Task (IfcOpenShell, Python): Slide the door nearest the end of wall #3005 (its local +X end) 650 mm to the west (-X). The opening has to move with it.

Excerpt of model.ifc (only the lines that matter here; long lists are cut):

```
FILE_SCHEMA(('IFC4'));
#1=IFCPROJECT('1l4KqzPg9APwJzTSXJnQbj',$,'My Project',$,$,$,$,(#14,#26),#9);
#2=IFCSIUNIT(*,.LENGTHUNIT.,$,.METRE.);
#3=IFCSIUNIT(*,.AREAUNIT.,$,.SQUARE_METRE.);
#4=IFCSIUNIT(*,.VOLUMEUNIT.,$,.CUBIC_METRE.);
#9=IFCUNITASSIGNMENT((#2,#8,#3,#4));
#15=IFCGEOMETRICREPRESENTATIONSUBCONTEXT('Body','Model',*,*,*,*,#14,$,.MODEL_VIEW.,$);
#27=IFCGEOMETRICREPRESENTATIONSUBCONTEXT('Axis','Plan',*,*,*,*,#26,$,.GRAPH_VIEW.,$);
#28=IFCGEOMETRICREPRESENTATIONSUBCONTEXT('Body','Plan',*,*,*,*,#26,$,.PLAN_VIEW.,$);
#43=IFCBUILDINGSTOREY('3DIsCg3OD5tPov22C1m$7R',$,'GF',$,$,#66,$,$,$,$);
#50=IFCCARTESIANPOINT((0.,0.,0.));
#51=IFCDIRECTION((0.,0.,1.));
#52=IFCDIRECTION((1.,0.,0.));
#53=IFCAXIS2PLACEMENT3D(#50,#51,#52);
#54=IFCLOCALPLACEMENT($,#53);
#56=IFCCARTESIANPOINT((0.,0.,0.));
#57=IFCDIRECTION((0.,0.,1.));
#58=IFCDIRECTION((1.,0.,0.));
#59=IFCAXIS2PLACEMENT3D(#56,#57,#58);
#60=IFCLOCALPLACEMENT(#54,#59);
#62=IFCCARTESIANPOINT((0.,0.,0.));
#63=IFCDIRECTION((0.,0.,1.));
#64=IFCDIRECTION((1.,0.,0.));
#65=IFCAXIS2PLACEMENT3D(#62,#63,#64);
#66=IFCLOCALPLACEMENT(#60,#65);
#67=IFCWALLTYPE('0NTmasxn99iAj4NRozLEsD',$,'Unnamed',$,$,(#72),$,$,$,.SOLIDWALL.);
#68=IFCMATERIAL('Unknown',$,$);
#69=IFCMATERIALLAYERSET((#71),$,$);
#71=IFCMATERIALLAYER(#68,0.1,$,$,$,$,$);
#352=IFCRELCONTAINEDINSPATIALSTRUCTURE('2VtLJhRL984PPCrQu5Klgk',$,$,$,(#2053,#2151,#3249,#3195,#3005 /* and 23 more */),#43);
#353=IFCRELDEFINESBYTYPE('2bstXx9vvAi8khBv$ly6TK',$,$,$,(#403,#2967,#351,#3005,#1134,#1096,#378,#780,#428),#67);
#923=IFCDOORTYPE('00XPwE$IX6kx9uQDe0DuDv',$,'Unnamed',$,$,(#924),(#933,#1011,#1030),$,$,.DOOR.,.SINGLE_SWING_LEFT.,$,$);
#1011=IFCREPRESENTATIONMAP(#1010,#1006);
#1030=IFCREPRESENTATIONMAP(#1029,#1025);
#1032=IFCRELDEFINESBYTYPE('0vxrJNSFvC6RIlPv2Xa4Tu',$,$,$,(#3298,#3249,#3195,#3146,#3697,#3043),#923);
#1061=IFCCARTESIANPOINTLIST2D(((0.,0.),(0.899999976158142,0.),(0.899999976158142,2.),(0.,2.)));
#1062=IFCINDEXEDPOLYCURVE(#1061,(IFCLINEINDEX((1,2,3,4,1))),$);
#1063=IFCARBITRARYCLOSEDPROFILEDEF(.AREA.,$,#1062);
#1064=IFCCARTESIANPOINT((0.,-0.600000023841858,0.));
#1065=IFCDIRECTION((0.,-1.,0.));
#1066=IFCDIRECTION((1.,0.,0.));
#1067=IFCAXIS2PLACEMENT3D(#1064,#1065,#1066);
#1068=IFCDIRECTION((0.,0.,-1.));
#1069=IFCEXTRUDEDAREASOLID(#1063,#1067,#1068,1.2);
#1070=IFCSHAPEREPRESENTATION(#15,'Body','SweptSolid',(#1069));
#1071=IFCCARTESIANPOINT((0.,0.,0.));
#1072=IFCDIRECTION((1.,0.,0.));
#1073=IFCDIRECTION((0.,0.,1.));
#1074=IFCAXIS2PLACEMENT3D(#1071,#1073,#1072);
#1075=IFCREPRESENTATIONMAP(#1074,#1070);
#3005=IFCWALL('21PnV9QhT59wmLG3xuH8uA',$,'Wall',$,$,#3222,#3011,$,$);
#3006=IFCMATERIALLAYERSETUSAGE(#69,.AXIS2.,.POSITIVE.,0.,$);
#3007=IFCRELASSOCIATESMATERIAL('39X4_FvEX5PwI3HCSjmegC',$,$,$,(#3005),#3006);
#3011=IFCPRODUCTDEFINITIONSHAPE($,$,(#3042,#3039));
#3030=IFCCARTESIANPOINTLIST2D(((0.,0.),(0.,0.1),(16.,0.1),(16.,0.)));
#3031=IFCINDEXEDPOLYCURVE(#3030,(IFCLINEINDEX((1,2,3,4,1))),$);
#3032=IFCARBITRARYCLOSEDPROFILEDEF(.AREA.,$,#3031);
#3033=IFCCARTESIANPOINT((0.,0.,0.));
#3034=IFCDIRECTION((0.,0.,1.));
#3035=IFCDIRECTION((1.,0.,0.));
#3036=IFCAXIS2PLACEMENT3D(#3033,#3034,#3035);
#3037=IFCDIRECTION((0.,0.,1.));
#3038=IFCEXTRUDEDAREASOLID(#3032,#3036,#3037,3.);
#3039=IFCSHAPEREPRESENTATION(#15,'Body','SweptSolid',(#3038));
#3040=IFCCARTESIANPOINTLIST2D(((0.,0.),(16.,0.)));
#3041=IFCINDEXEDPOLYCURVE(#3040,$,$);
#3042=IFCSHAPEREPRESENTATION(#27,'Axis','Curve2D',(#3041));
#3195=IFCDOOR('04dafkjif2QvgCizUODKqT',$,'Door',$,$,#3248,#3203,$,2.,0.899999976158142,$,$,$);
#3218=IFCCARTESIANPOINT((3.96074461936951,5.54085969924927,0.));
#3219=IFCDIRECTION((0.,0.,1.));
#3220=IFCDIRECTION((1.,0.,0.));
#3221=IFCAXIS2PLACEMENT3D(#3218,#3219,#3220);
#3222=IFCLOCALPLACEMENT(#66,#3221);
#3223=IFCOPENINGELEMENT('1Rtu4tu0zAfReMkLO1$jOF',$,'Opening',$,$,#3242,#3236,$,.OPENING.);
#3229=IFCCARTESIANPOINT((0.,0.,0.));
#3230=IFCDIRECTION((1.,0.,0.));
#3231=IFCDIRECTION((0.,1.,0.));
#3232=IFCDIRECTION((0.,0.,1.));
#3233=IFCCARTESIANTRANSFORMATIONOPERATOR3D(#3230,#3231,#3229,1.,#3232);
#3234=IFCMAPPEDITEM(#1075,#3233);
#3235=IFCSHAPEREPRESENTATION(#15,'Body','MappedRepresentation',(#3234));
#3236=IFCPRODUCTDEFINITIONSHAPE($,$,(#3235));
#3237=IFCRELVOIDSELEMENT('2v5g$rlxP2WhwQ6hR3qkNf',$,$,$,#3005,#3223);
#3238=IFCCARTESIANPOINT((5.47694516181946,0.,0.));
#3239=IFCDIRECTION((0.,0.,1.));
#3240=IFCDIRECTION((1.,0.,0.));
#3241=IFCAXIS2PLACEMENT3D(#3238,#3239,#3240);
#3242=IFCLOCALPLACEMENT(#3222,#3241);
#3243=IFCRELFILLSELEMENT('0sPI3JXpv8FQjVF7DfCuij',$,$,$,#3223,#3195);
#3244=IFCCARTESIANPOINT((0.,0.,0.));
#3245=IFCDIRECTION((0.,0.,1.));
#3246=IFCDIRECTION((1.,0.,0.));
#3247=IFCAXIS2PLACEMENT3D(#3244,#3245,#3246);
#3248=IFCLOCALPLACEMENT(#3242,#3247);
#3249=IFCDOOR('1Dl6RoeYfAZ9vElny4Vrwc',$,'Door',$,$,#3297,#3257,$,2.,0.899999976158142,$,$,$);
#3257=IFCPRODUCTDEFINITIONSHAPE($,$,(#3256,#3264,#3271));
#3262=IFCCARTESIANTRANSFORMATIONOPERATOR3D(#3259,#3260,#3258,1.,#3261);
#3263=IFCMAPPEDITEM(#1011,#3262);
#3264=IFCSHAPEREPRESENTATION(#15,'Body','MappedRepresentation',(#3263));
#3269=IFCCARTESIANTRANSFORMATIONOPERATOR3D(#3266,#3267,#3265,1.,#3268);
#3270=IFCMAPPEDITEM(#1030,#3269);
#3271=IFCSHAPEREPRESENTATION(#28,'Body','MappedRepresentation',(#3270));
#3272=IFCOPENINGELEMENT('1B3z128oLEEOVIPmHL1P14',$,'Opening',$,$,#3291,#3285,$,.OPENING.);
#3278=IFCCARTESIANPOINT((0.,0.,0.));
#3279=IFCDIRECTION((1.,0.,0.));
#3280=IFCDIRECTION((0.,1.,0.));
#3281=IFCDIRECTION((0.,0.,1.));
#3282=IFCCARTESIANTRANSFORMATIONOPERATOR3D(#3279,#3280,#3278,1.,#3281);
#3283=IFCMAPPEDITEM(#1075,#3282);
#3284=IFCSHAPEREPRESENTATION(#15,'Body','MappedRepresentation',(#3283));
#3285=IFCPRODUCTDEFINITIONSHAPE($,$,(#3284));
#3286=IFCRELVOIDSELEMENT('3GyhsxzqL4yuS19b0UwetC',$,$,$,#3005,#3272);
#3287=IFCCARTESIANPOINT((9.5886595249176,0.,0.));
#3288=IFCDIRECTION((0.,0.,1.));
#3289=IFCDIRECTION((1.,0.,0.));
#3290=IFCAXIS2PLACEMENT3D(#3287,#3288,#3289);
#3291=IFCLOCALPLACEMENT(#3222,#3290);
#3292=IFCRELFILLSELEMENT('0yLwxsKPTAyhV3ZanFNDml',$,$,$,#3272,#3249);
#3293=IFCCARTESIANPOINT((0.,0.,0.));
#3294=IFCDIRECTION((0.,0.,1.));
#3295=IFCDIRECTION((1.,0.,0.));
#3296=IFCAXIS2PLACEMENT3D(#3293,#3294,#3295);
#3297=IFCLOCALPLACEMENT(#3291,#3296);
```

```python
import ifcopenshell
import ifcopenshell.api.geometry
import ifcopenshell.util.placement

model = ifcopenshell.open("model.ifc")

door = model.by_guid("1Dl6RoeYfAZ9vElny4Vrwc")
opening = door.FillsVoids[0].RelatingOpeningElement
wall = opening.VoidsElements[0].RelatingBuildingElement

wall_matrix = ifcopenshell.util.placement.get_local_placement(wall.ObjectPlacement)
shift = wall_matrix[:3, 0] * -0.65
before = ifcopenshell.util.placement.get_local_placement(door.ObjectPlacement)[:3, 3].copy()

# The door is placed relative to its opening, so it follows when the opening moves.
matrix = ifcopenshell.util.placement.get_local_placement(opening.ObjectPlacement)
matrix[:3, 3] += shift
ifcopenshell.api.geometry.edit_object_placement(
    model, product=opening, matrix=matrix, is_si=False, should_transform_children=True
)

after = ifcopenshell.util.placement.get_local_placement(door.ObjectPlacement)[:3, 3]
print("door moved by", (after - before).round(3) + 0.0)

model.write("model_rev.ifc")
```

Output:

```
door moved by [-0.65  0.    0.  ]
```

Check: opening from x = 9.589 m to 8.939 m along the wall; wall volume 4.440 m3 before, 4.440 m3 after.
